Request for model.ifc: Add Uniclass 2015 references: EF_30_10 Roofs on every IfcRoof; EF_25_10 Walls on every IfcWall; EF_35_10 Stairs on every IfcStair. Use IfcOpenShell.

First a look at what the model holds.

```python
import ifcopenshell

model = ifcopenshell.open("model.ifc")
print(model.schema)
print("classifications:", [c.Name for c in model.by_type("IfcClassification")])
for ifc_class in ("IfcDoor", "IfcRoof", "IfcStair", "IfcWall", "IfcWindow"):
    print(ifc_class, len(model.by_type(ifc_class)))
```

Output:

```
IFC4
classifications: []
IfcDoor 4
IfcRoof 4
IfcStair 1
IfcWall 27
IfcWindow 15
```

```python
import ifcopenshell
import ifcopenshell.api.classification

model = ifcopenshell.open("model.ifc")

system = ifcopenshell.api.classification.add_classification(model, classification="Uniclass 2015")

codes = {
    "IfcRoof": ("EF_30_10", "Roofs"),
    "IfcWall": ("EF_25_10", "Walls"),
    "IfcStair": ("EF_35_10", "Stairs"),
}
for ifc_class, (code, name) in codes.items():
    products = model.by_type(ifc_class)
    ifcopenshell.api.classification.add_reference(
        model, products=products, classification=system, identification=code, name=name
    )
    print(code, len(products))

model.write("model_updated.ifc")
```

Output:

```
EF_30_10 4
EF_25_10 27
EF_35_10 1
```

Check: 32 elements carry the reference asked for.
